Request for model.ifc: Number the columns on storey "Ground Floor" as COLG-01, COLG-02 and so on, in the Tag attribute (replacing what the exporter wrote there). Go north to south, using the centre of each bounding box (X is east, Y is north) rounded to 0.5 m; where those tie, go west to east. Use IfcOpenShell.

First a look at what the model holds.

```python
import ifcopenshell
import ifcopenshell.util.element
import ifcopenshell.util.placement

model = ifcopenshell.open("model.ifc")
print(model.schema)
storey = next(s for s in model.by_type("IfcBuildingStorey") if s.Name == "Ground Floor")
columns = [e for e in ifcopenshell.util.element.get_decomposition(storey) if e.is_a("IfcColumn")]
for e in sorted(columns, key=lambda e: e.id()):
    origin = ifcopenshell.util.placement.get_local_placement(e.ObjectPlacement)[:3, 3]
    print(e.id(), e.Tag, e.Name, origin.round(2) + 0.0, sep=" | ")
```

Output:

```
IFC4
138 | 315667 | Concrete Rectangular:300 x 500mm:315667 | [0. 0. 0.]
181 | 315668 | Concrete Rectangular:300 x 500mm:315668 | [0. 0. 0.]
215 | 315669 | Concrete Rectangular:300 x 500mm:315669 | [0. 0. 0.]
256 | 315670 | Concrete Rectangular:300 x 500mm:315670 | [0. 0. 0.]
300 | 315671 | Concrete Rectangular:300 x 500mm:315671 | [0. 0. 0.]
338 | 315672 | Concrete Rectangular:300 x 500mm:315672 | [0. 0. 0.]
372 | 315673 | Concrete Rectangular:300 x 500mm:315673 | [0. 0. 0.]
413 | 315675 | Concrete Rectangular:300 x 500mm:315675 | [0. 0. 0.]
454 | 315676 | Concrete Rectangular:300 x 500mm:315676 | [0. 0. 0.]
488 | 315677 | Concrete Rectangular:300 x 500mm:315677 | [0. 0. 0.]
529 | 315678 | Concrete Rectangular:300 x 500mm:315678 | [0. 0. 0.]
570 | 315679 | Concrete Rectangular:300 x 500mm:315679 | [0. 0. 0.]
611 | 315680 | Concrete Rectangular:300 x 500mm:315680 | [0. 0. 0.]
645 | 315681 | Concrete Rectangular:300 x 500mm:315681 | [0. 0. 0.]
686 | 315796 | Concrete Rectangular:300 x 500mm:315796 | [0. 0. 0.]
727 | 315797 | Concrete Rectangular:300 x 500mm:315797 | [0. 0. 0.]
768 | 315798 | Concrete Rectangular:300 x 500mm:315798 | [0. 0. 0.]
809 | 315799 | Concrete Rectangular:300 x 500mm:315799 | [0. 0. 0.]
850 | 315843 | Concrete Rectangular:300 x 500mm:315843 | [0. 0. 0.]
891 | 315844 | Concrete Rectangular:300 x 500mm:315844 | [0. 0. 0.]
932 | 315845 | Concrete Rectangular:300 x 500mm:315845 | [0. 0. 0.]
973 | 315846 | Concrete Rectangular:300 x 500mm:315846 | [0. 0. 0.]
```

```python
import ifcopenshell
import ifcopenshell.geom
import ifcopenshell.util.element
import ifcopenshell.util.shape

model = ifcopenshell.open("model.ifc")
settings = ifcopenshell.geom.settings()
settings.set("use-world-coords", True)


def centre(element):
    shape = ifcopenshell.geom.create_shape(settings, element)
    return ifcopenshell.util.shape.get_bbox_centroid(shape.geometry)


storey = next(s for s in model.by_type("IfcBuildingStorey") if s.Name == "Ground Floor")
columns = [e for e in ifcopenshell.util.element.get_decomposition(storey) if e.is_a("IfcColumn")]

# Insertion points can sit at a corner or the storey origin, so sort by the geometry (in metres).
centres = {e: centre(e) for e in columns}
columns.sort(key=lambda e: (-round(centres[e][1] / 0.5), centres[e][0]))

for i, e in enumerate(columns, start=1):
    number = f"COLG-{i:02d}"
    e.Tag = number
    print(e.id(), number)

model.write("model_v2.ifc")
```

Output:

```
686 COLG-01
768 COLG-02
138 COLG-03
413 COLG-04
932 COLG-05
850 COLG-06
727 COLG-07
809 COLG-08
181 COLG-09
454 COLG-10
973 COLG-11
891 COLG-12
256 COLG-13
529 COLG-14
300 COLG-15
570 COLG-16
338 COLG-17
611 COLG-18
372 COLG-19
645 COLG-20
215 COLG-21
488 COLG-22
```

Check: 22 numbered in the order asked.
